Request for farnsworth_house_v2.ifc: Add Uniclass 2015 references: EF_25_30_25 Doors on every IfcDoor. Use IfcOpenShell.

First a look at what the model holds.

```python
import ifcopenshell

model = ifcopenshell.open("farnsworth_house_v2.ifc")
print(model.schema)
print("classifications:", [c.Name for c in model.by_type("IfcClassification")])
for ifc_class in ("IfcDoor", "IfcRoof", "IfcStair", "IfcWall", "IfcWindow"):
    print(ifc_class, len(model.by_type(ifc_class)))
```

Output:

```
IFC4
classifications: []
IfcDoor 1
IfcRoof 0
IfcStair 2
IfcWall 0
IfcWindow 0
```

```python
import ifcopenshell
import ifcopenshell.api.classification

model = ifcopenshell.open("farnsworth_house_v2.ifc")

system = ifcopenshell.api.classification.add_classification(model, classification="Uniclass 2015")

codes = {
    "IfcDoor": ("EF_25_30_25", "Doors"),
}
for ifc_class, (code, name) in codes.items():
    products = model.by_type(ifc_class)
    ifcopenshell.api.classification.add_reference(
        model, products=products, classification=system, identification=code, name=name
    )
    print(code, len(products))

model.write("farnsworth_house_v2_rev.ifc")
```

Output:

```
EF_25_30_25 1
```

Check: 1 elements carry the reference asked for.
